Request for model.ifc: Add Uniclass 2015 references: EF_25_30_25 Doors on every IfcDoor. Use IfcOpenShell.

First a look at what the model holds.

```python
import ifcopenshell

model = ifcopenshell.open("model.ifc")
print(model.schema)
print("classifications:", [c.Name for c in model.by_type("IfcClassification")])
for ifc_class in ("IfcDoor", "IfcRoof", "IfcStair", "IfcWall", "IfcWindow"):
    print(ifc_class, len(model.by_type(ifc_class)))
```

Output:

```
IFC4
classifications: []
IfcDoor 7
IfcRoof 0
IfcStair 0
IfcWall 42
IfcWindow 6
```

```python
import ifcopenshell
import ifcopenshell.api.classification

model = ifcopenshell.open("model.ifc")

system = ifcopenshell.api.classification.add_classification(model, classification="Uniclass 2015")

codes = {
    "IfcDoor": ("EF_25_30_25", "Doors"),
}
for ifc_class, (code, name) in codes.items():
    products = model.by_type(ifc_class)
    ifcopenshell.api.classification.add_reference(
        model, products=products, classification=system, identification=code, name=name
    )
    print(code, len(products))

model.write("model_updated.ifc")
```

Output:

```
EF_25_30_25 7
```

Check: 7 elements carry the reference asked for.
